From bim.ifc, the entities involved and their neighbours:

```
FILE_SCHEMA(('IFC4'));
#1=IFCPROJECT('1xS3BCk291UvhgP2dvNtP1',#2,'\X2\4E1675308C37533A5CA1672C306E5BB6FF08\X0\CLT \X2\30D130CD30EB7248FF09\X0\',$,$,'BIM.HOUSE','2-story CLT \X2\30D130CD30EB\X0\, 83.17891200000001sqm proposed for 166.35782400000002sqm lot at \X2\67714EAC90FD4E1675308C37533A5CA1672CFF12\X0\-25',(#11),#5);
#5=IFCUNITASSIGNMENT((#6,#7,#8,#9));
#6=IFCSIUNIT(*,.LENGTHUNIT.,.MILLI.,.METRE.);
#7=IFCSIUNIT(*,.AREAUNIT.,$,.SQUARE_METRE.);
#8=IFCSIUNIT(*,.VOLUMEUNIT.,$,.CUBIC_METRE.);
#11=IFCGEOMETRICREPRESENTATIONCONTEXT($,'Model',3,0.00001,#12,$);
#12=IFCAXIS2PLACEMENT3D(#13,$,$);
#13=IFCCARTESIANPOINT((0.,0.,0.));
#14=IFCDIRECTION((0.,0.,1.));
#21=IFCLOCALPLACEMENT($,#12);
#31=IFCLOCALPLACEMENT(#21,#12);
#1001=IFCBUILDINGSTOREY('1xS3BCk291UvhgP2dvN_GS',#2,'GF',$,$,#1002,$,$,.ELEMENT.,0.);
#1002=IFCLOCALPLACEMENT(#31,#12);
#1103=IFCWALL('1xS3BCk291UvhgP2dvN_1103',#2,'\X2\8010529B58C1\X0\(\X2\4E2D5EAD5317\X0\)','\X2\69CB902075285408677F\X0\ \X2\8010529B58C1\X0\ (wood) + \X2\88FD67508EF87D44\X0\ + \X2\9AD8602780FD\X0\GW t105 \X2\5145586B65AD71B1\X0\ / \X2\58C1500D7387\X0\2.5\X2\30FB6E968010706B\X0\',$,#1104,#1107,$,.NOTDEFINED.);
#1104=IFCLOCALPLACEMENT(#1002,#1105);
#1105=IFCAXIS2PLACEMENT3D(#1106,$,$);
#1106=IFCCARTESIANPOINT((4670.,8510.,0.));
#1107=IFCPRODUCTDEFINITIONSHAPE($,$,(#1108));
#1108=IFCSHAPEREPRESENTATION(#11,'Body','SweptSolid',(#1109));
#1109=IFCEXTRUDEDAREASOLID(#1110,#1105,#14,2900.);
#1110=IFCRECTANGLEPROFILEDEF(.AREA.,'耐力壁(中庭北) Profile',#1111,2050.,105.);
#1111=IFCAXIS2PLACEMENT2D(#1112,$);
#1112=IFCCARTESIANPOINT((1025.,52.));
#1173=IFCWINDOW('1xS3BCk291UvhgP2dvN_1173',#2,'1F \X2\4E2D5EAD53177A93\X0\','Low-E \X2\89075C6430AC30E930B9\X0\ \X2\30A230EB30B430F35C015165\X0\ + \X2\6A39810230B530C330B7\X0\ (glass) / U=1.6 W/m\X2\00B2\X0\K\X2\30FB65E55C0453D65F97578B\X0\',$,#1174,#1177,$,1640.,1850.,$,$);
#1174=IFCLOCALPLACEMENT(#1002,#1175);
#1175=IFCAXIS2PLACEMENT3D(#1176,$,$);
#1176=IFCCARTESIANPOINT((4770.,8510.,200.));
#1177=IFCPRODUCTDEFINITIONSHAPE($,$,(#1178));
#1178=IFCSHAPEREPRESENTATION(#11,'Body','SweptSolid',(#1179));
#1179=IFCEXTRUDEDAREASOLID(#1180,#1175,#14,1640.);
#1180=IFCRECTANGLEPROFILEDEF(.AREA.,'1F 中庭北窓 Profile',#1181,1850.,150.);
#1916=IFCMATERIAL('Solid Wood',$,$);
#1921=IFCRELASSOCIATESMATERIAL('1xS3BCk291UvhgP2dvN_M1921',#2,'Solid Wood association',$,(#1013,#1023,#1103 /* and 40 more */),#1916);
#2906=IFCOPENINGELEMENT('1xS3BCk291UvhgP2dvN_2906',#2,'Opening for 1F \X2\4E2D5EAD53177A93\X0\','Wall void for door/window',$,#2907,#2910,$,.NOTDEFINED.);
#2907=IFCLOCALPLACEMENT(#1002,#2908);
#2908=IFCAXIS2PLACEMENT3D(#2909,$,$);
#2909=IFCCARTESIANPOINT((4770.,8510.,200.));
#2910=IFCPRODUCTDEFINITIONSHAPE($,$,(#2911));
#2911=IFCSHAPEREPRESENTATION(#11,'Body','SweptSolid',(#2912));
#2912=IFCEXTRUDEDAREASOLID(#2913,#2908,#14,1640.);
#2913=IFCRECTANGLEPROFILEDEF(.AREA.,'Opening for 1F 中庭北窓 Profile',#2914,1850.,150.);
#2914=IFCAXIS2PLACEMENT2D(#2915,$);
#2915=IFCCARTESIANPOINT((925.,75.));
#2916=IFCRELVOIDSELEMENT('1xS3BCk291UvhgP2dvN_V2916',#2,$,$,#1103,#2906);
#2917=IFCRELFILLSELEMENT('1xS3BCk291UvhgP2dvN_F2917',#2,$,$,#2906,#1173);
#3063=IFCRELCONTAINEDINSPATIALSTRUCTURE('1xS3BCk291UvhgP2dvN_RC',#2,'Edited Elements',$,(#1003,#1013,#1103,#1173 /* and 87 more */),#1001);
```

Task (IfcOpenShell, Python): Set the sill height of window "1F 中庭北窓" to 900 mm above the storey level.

```python
import numpy as np
import ifcopenshell
import ifcopenshell.api.geometry
import ifcopenshell.geom
import ifcopenshell.util.element
import ifcopenshell.util.placement
import ifcopenshell.util.shape
import ifcopenshell.util.unit

model = ifcopenshell.open("bim.ifc")
unit_scale = ifcopenshell.util.unit.calculate_unit_scale(model)

window = model.by_guid("1xS3BCk291UvhgP2dvN_1173")
opening = window.FillsVoids[0].RelatingOpeningElement
storey = ifcopenshell.util.element.get_container(window, ifc_class="IfcBuildingStorey")
level = ifcopenshell.util.placement.get_local_placement(storey.ObjectPlacement)[2, 3]

# The opening's origin need not be at the sill, so measure its lowest point.
shape = ifcopenshell.geom.create_shape(ifcopenshell.geom.settings(), opening)
bottom = ifcopenshell.util.shape.get_shape_bottom_elevation(shape, shape.geometry) / unit_scale
dz = level + 900.0 - bottom

shift = np.array([0.0, 0.0, dz])
# The window is not placed relative to its opening, so move both.
for product in (opening, window):
    matrix = ifcopenshell.util.placement.get_local_placement(product.ObjectPlacement)
    matrix[:3, 3] += shift
    ifcopenshell.api.geometry.edit_object_placement(model, product=product, matrix=matrix, is_si=False)

print(f"moved by {dz * unit_scale:+.3f} m")

model.write("bim_edited.ifc")
```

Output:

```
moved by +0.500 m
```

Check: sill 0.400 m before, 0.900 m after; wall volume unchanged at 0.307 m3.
